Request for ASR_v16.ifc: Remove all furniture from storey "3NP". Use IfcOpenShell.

First a look at what the model holds.

```python
import ifcopenshell
import ifcopenshell.util.element

model = ifcopenshell.open("ASR_v16.ifc")
print(model.schema)
storey = next(s for s in model.by_type("IfcBuildingStorey") if s.Name == "3NP")
furniture = [e for e in ifcopenshell.util.element.get_decomposition(storey) if e.is_a("IfcFurnishingElement")]
seen = {}
for e in furniture:
    element_type = ifcopenshell.util.element.get_type(e)
    name = element_type.Name if element_type not in (None, e) else None
    seen[name] = seen.get(name, 0) + 1
for name, count in sorted(seen.items(), key=str):
    print(count, "x", name)
```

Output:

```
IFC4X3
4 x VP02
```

```python
import ifcopenshell
import ifcopenshell.api.root
import ifcopenshell.util.element

model = ifcopenshell.open("ASR_v16.ifc")

storey = next(s for s in model.by_type("IfcBuildingStorey") if s.Name == "3NP")
furniture = [e for e in ifcopenshell.util.element.get_decomposition(storey) if e.is_a("IfcFurnishingElement")]

for e in furniture:
    ifcopenshell.api.root.remove_product(model, product=e)
print(len(furniture), "removed")

model.write("ASR_v16_v2.ifc")
```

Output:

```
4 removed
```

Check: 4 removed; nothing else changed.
